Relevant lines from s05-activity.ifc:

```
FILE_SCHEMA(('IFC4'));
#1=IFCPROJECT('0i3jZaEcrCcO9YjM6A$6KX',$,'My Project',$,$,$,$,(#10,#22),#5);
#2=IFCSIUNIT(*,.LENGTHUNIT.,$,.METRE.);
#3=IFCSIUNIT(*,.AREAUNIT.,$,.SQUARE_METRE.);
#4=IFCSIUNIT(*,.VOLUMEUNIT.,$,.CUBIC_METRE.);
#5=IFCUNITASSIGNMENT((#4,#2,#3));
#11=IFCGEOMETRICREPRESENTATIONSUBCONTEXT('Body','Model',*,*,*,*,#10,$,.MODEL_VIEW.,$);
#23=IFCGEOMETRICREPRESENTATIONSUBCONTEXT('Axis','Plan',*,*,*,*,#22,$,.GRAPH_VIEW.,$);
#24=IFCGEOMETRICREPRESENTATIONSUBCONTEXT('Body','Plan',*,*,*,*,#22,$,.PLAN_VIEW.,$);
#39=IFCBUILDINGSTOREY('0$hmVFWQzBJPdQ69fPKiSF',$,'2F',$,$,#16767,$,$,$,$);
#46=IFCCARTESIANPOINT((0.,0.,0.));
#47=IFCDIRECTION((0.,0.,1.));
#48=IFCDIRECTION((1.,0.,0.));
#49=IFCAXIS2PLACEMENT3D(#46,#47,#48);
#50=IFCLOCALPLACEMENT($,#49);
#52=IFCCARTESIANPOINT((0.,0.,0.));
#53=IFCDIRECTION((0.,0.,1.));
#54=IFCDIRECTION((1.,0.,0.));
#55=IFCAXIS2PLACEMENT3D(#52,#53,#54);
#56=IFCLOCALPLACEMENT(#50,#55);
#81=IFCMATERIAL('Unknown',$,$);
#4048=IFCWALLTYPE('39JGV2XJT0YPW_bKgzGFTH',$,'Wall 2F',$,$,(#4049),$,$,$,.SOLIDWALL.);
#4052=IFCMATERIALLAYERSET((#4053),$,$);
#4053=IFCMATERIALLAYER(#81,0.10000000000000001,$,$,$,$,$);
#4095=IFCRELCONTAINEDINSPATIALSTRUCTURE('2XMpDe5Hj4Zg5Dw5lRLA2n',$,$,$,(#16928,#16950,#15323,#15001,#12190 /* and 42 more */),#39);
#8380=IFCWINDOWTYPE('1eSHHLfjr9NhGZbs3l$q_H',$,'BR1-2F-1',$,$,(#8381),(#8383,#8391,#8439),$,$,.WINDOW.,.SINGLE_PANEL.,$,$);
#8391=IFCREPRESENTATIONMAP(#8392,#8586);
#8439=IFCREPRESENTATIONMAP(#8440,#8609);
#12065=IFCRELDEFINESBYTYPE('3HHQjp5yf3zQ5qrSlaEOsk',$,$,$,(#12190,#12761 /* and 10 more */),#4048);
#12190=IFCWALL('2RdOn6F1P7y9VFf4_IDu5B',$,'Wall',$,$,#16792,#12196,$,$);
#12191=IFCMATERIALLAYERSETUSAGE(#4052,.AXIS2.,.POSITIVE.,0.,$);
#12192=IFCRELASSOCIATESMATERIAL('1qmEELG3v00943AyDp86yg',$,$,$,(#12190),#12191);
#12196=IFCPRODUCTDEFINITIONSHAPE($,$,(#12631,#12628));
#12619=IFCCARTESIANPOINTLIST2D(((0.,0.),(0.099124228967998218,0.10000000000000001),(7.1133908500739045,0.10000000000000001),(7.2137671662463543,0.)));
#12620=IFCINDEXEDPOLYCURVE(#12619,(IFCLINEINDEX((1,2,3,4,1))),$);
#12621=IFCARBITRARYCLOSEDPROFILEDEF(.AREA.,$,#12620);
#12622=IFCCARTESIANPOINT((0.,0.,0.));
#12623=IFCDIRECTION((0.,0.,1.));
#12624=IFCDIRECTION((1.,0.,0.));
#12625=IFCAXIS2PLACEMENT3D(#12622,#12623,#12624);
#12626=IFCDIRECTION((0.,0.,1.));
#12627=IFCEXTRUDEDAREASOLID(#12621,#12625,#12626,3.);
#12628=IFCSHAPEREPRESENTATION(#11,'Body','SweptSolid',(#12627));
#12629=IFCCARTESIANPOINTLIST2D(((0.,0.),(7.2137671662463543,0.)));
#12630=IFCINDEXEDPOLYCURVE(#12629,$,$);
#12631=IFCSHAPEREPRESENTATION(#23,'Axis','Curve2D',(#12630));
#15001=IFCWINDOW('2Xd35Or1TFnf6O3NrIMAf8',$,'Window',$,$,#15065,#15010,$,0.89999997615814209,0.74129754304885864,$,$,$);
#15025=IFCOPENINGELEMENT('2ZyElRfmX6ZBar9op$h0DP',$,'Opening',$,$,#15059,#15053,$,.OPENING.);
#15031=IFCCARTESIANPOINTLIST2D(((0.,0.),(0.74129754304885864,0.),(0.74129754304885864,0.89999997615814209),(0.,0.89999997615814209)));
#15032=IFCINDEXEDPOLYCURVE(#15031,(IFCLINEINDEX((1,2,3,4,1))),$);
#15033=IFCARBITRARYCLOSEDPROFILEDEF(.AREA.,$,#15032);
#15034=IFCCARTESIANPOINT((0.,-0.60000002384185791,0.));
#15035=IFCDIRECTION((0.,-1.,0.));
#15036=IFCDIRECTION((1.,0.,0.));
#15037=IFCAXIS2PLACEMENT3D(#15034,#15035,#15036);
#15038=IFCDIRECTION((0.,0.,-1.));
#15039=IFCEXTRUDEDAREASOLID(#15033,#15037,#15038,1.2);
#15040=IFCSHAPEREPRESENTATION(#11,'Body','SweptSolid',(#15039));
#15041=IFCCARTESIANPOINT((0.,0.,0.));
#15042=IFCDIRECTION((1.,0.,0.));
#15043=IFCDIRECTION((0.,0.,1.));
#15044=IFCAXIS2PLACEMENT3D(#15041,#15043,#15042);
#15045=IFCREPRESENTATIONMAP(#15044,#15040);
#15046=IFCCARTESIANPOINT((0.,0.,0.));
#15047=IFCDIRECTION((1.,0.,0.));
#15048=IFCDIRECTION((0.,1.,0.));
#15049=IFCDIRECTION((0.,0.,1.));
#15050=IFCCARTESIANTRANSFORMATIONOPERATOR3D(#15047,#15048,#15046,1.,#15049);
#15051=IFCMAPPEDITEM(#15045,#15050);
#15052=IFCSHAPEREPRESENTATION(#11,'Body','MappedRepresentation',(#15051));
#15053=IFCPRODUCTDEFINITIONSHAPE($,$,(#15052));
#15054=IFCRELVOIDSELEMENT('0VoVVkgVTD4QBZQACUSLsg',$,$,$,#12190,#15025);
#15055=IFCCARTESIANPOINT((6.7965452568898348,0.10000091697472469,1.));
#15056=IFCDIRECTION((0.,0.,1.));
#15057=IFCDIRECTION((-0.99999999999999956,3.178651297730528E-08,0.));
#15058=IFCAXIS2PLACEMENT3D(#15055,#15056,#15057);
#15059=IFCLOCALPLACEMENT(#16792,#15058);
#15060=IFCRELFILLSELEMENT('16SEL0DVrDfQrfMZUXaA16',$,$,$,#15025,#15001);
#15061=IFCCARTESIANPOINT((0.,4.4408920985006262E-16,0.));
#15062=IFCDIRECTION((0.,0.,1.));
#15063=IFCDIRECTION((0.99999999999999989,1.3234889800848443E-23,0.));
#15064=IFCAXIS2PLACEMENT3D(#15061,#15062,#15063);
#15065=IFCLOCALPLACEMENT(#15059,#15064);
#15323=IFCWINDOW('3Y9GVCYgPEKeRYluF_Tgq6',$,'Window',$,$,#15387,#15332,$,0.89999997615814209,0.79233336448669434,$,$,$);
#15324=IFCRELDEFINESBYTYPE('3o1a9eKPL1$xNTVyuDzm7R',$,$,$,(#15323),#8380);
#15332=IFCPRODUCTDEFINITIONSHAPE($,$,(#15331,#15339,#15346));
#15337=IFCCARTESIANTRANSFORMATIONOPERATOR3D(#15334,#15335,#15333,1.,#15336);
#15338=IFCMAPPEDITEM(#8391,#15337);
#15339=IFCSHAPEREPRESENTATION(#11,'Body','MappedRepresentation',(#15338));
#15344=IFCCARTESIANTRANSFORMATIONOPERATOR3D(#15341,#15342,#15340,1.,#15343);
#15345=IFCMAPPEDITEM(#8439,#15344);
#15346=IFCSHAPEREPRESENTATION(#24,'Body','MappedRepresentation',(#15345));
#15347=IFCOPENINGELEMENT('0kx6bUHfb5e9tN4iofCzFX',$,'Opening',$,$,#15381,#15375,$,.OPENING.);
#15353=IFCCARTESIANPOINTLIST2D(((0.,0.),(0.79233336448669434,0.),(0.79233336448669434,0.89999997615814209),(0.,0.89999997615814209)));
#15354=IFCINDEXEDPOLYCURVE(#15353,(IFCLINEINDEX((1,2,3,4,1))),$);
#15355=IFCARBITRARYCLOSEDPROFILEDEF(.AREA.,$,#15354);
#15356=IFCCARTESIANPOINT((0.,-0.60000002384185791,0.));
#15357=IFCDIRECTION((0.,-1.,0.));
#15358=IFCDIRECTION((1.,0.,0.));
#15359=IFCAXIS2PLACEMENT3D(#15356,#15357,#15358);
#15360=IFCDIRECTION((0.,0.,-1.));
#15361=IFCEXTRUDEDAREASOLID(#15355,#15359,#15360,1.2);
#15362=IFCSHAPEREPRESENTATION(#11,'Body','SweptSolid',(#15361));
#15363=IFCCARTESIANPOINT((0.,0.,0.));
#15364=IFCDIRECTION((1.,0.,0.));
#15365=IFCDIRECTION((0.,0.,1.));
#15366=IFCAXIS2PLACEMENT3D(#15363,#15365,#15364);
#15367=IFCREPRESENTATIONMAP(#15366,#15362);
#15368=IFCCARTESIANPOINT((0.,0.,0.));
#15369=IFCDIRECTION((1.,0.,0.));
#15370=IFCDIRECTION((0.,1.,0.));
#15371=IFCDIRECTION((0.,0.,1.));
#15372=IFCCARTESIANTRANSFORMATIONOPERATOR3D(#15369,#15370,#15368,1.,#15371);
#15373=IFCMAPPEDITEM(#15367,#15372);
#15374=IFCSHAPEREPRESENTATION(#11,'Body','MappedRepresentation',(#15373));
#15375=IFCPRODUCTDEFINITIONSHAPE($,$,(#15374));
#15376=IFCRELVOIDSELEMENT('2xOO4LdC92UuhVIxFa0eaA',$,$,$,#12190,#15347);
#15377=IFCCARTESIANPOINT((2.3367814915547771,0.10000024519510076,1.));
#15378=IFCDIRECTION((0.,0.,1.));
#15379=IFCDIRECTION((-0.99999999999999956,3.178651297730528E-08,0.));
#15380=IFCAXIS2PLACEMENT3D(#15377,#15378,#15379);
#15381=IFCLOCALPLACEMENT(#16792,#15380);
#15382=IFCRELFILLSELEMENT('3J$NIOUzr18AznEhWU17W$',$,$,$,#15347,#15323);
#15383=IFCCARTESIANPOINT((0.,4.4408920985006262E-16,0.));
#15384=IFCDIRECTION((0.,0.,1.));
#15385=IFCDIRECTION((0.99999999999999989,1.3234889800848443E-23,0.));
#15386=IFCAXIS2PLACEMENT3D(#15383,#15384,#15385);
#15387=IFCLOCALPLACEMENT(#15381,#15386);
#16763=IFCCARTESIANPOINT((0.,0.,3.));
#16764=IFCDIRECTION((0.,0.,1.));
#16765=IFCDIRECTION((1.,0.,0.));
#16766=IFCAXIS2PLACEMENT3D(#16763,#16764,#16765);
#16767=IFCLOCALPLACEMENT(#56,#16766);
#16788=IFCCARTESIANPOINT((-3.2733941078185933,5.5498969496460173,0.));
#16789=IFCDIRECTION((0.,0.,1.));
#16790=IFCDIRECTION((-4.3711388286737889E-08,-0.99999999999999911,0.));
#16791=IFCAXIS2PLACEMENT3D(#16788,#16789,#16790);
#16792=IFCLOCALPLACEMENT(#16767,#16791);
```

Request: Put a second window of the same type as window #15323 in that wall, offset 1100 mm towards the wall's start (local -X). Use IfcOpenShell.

```python
import ifcopenshell
import ifcopenshell.api.feature
import ifcopenshell.api.geometry
import ifcopenshell.api.root
import ifcopenshell.geom
import ifcopenshell.util.element
import ifcopenshell.util.placement
import ifcopenshell.util.shape

model = ifcopenshell.open("s05-activity.ifc")
settings = ifcopenshell.geom.settings()


def volume(element):
    """Net volume in cubic metres, openings subtracted."""
    shape = ifcopenshell.geom.create_shape(settings, element)
    return ifcopenshell.util.shape.get_volume(shape.geometry)


window = model.by_id(15323)
opening = window.FillsVoids[0].RelatingOpeningElement
wall = opening.VoidsElements[0].RelatingBuildingElement
before = volume(wall)
shift = ifcopenshell.util.placement.get_local_placement(wall.ObjectPlacement)[:3, 0] * -1.1

# copy_class copies the void relationship, type, container and properties, but no geometry.
new_opening = ifcopenshell.api.root.copy_class(model, product=opening)
new_opening.Representation = ifcopenshell.util.element.copy_deep(
    model, opening.Representation, exclude=["IfcGeometricRepresentationContext", "IfcRepresentationMap"]
)
new_window = ifcopenshell.api.root.copy_class(model, product=window)
new_window.Representation = ifcopenshell.util.element.copy_deep(
    model, window.Representation, exclude=["IfcGeometricRepresentationContext", "IfcRepresentationMap"]
)
ifcopenshell.api.feature.add_filling(model, opening=new_opening, element=new_window)

for old, new in ((opening, new_opening), (window, new_window)):
    matrix = ifcopenshell.util.placement.get_local_placement(old.ObjectPlacement)
    matrix[:3, 3] += shift
    ifcopenshell.api.geometry.edit_object_placement(model, product=new, matrix=matrix, is_si=False)

after = volume(wall)

print(f"wall volume {before:.3f} -> {after:.3f} m3")

model.write("s05-activity-out.ifc")
```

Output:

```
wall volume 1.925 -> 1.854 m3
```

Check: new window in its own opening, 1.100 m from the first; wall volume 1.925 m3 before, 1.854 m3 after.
